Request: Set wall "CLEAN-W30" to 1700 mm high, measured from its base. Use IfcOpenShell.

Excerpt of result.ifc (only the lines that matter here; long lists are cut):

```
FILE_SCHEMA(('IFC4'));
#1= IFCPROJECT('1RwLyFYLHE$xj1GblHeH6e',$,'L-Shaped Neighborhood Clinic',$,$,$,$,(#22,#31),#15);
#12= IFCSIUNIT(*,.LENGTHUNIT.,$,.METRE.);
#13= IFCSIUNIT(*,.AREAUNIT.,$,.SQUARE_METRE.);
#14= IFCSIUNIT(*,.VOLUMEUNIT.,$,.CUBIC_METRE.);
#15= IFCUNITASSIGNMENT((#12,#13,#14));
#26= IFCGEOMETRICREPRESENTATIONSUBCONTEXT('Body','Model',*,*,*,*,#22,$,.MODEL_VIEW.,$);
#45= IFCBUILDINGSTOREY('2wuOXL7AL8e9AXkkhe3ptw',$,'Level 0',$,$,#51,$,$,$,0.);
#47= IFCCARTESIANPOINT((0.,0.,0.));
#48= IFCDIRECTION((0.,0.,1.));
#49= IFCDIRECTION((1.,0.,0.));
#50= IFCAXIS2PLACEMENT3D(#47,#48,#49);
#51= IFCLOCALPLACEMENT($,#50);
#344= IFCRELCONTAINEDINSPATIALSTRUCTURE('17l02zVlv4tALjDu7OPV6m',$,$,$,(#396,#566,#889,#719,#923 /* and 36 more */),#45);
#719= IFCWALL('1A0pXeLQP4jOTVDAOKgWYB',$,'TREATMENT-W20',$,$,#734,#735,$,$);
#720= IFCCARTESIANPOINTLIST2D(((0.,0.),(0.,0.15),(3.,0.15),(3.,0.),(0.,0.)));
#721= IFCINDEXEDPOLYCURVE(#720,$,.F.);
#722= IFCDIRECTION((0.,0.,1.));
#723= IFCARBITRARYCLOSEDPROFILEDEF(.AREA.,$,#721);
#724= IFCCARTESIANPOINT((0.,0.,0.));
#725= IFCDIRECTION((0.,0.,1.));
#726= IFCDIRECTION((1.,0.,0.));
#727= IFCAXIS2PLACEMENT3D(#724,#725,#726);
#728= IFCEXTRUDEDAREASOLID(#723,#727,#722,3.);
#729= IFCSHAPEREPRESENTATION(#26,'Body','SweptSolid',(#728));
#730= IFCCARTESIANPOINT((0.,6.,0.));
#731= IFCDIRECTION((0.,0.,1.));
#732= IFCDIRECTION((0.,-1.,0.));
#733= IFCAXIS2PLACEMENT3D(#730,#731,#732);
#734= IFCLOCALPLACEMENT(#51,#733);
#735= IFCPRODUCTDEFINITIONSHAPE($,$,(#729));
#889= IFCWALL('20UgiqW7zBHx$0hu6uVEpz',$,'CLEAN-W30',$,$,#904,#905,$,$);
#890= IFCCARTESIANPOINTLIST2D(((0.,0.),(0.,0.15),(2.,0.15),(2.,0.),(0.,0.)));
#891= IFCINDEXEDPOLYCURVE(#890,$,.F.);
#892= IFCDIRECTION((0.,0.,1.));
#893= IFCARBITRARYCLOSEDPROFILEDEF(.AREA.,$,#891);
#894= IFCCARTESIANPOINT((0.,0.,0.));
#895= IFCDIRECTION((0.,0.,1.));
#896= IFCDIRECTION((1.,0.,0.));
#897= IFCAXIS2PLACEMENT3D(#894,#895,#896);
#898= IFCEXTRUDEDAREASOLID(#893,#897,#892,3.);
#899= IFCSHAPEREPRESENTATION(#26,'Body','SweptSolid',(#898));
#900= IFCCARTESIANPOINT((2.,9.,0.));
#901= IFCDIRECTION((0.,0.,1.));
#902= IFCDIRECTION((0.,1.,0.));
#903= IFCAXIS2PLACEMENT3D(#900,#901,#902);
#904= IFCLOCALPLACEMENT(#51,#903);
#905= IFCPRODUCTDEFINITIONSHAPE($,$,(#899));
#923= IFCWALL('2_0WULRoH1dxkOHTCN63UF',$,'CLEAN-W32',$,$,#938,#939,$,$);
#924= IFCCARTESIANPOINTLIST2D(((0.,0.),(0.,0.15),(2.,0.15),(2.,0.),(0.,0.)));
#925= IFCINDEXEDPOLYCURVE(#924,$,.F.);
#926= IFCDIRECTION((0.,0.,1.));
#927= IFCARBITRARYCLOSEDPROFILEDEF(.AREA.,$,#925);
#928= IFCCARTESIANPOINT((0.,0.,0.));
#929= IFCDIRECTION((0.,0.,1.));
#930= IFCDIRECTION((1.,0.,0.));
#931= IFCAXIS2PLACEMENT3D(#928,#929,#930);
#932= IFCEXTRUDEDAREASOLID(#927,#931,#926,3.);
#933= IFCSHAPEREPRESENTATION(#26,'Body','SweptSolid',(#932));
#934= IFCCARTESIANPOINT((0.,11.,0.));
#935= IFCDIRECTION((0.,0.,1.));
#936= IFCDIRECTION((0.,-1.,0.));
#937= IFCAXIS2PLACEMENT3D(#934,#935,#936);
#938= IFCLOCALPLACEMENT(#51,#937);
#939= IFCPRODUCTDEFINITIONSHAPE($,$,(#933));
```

```python
import ifcopenshell
import ifcopenshell.geom
import ifcopenshell.util.representation
import ifcopenshell.util.shape
import ifcopenshell.util.unit

model = ifcopenshell.open("result.ifc")
unit_scale = ifcopenshell.util.unit.calculate_unit_scale(model)
settings = ifcopenshell.geom.settings()


def volume(element):
    """Net volume in cubic metres, openings subtracted."""
    shape = ifcopenshell.geom.create_shape(settings, element)
    return ifcopenshell.util.shape.get_volume(shape.geometry)


wall = model.by_guid("20UgiqW7zBHx$0hu6uVEpz")
before = volume(wall)

body = ifcopenshell.util.representation.get_representation(wall, "Model", "Body")
solid = body.Items[0]
old_height = solid.Depth
solid.Depth = 1.7 / unit_scale
after = volume(wall)

print(f"height {old_height:g} -> {solid.Depth:g}, volume {before:.3f} -> {after:.3f} m3")

model.write("result_updated.ifc")
```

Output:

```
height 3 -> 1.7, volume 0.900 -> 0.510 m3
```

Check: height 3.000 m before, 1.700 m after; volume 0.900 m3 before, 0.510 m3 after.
